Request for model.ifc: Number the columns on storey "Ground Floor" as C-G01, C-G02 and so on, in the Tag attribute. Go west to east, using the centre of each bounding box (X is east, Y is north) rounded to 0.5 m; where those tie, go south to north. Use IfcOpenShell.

First a look at what the model holds.

```python
import ifcopenshell
import ifcopenshell.util.element
import ifcopenshell.util.placement

model = ifcopenshell.open("model.ifc")
print(model.schema)
storey = next(s for s in model.by_type("IfcBuildingStorey") if s.Name == "Ground Floor")
columns = [e for e in ifcopenshell.util.element.get_decomposition(storey) if e.is_a("IfcColumn")]
for e in sorted(columns, key=lambda e: e.id()):
    origin = ifcopenshell.util.placement.get_local_placement(e.ObjectPlacement)[:3, 3]
    print(e.id(), e.Tag, e.Name, origin.round(2) + 0.0, sep=" | ")
```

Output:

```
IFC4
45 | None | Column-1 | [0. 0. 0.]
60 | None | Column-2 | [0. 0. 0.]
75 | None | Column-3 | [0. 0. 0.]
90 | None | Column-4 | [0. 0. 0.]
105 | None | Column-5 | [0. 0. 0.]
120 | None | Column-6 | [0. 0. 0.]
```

```python
import ifcopenshell
import ifcopenshell.geom
import ifcopenshell.util.element
import ifcopenshell.util.shape

model = ifcopenshell.open("model.ifc")
settings = ifcopenshell.geom.settings()
settings.set("use-world-coords", True)


def centre(element):
    shape = ifcopenshell.geom.create_shape(settings, element)
    return ifcopenshell.util.shape.get_bbox_centroid(shape.geometry)


storey = next(s for s in model.by_type("IfcBuildingStorey") if s.Name == "Ground Floor")
columns = [e for e in ifcopenshell.util.element.get_decomposition(storey) if e.is_a("IfcColumn")]

# Insertion points can sit at a corner or the storey origin, so sort by the geometry (in metres).
centres = {e: centre(e) for e in columns}
columns.sort(key=lambda e: (round(centres[e][0] / 0.5), centres[e][1]))

for i, e in enumerate(columns, start=1):
    number = f"C-G{i:02d}"
    e.Tag = number
    print(e.id(), number)

model.write("model_v2.ifc")
```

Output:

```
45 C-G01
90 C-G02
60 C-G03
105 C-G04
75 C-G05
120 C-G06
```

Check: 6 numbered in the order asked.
